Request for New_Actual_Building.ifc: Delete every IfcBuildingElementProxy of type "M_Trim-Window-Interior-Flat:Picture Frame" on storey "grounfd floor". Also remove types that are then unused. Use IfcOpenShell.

First a look at what the model holds.

```python
import ifcopenshell
import ifcopenshell.util.element

model = ifcopenshell.open("New_Actual_Building.ifc")
print(model.schema)
storey = next(s for s in model.by_type("IfcBuildingStorey") if s.Name == "grounfd floor")
proxies = [e for e in ifcopenshell.util.element.get_decomposition(storey) if e.is_a("IfcBuildingElementProxy")]
seen = {}
for e in proxies:
    element_type = ifcopenshell.util.element.get_type(e)
    name = element_type.Name if element_type not in (None, e) else None
    seen[name] = seen.get(name, 0) + 1
for name, count in sorted(seen.items(), key=str):
    print(count, "x", name)
```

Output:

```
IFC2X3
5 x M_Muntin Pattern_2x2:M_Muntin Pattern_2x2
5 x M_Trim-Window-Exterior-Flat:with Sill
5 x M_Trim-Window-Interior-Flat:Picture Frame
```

```python
import ifcopenshell
import ifcopenshell.api.root
import ifcopenshell.util.element

model = ifcopenshell.open("New_Actual_Building.ifc")

storey = next(s for s in model.by_type("IfcBuildingStorey") if s.Name == "grounfd floor")
proxies = [e for e in ifcopenshell.util.element.get_decomposition(storey) if e.is_a("IfcBuildingElementProxy")]
targets = [e for e in proxies if (t := ifcopenshell.util.element.get_type(e)) not in (None, e) and t.Name == "M_Trim-Window-Interior-Flat:Picture Frame"]
types = {ifcopenshell.util.element.get_type(e) for e in targets} - {None, *targets}

for e in targets:
    ifcopenshell.api.root.remove_product(model, product=e)
print(len(targets), "removed")

unused = [t for t in types if not ifcopenshell.util.element.get_types(t)]
for t in unused:
    ifcopenshell.api.root.remove_product(model, product=t)
print(len(unused), "unused types removed")

model.write("New_Actual_Building-out.ifc")
```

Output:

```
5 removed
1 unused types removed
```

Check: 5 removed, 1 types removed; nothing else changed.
